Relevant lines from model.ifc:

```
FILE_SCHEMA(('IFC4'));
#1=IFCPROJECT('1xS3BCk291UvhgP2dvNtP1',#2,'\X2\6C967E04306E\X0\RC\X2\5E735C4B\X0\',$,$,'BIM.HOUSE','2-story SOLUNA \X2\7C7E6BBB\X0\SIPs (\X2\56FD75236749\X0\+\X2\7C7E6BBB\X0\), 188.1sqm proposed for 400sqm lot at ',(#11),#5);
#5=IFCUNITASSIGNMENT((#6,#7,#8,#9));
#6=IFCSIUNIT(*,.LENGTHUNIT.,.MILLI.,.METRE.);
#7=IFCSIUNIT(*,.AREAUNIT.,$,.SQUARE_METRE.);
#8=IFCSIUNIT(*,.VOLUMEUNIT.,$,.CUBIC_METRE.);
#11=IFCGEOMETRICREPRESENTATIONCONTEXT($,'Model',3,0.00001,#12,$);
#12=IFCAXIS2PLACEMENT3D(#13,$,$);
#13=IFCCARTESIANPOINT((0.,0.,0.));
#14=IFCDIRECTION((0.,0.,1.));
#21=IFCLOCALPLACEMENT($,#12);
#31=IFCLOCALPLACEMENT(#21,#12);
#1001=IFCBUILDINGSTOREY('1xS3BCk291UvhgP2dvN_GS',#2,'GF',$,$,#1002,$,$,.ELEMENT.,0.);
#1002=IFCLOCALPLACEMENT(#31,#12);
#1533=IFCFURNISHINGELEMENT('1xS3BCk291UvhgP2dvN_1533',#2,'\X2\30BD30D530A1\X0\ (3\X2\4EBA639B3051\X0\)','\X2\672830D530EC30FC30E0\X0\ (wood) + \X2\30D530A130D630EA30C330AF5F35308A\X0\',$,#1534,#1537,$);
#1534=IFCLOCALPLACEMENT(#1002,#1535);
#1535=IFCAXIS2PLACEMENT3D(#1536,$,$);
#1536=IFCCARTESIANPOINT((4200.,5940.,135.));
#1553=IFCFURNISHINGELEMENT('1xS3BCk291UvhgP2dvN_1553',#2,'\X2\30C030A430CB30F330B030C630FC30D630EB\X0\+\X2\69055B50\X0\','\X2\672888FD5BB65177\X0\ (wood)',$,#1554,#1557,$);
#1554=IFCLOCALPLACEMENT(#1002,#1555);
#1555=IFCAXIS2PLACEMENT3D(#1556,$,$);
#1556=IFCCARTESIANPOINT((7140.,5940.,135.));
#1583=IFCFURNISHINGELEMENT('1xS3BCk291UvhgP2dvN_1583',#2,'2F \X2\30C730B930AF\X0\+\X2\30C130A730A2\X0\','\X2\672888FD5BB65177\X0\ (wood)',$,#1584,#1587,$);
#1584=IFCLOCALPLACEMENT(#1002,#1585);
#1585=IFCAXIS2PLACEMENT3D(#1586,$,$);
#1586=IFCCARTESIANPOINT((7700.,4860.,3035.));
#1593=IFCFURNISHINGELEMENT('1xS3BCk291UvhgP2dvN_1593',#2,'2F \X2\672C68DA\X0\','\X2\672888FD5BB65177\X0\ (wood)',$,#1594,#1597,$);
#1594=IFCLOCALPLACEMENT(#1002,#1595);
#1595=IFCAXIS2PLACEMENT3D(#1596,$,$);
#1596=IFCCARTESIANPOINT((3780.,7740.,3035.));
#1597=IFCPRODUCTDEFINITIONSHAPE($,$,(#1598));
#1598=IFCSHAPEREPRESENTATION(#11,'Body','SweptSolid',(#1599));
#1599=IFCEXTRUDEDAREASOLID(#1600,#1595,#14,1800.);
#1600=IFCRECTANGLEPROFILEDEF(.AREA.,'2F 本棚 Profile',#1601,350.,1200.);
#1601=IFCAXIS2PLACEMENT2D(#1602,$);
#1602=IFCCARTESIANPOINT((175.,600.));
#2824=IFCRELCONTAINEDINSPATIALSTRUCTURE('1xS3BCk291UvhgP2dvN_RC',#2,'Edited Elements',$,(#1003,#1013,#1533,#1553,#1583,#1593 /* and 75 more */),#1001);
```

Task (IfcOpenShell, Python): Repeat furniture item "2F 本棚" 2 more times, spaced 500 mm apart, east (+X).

```python
import numpy as np
import ifcopenshell
import ifcopenshell.api.geometry
import ifcopenshell.api.root
import ifcopenshell.util.element
import ifcopenshell.util.placement

model = ifcopenshell.open("model.ifc")


def reuse_history(source, copy):
    """copy_class also copies each property set's owner history, people and application; keep the originals."""
    for rel in copy.IsDefinedBy:
        if rel.is_a("IfcRelDefinesByProperties") and (history := rel.RelatingPropertyDefinition.OwnerHistory):
            rel.RelatingPropertyDefinition.OwnerHistory = source.OwnerHistory
            ifcopenshell.util.element.remove_deep2(model, history)


source = model.by_guid("1xS3BCk291UvhgP2dvN_1593")
base = ifcopenshell.util.placement.get_local_placement(source.ObjectPlacement)
step = np.array([1.0, 0.0, 0.0]) * 500.0

for i in range(1, 3):
    copy = ifcopenshell.api.root.copy_class(model, product=source)
    copy.Representation = ifcopenshell.util.element.copy_deep(
        model, source.Representation, exclude=["IfcGeometricRepresentationContext", "IfcRepresentationMap"]
    )
    reuse_history(source, copy)
    matrix = base.copy()
    matrix[:3, 3] += i * step
    print("added at", matrix[:3, 3].round(3) + 0.0)
    ifcopenshell.api.geometry.edit_object_placement(model, product=copy, matrix=matrix, is_si=False)

model.write("model_v2.ifc")
```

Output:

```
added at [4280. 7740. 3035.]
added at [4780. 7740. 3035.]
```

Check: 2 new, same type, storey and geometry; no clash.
